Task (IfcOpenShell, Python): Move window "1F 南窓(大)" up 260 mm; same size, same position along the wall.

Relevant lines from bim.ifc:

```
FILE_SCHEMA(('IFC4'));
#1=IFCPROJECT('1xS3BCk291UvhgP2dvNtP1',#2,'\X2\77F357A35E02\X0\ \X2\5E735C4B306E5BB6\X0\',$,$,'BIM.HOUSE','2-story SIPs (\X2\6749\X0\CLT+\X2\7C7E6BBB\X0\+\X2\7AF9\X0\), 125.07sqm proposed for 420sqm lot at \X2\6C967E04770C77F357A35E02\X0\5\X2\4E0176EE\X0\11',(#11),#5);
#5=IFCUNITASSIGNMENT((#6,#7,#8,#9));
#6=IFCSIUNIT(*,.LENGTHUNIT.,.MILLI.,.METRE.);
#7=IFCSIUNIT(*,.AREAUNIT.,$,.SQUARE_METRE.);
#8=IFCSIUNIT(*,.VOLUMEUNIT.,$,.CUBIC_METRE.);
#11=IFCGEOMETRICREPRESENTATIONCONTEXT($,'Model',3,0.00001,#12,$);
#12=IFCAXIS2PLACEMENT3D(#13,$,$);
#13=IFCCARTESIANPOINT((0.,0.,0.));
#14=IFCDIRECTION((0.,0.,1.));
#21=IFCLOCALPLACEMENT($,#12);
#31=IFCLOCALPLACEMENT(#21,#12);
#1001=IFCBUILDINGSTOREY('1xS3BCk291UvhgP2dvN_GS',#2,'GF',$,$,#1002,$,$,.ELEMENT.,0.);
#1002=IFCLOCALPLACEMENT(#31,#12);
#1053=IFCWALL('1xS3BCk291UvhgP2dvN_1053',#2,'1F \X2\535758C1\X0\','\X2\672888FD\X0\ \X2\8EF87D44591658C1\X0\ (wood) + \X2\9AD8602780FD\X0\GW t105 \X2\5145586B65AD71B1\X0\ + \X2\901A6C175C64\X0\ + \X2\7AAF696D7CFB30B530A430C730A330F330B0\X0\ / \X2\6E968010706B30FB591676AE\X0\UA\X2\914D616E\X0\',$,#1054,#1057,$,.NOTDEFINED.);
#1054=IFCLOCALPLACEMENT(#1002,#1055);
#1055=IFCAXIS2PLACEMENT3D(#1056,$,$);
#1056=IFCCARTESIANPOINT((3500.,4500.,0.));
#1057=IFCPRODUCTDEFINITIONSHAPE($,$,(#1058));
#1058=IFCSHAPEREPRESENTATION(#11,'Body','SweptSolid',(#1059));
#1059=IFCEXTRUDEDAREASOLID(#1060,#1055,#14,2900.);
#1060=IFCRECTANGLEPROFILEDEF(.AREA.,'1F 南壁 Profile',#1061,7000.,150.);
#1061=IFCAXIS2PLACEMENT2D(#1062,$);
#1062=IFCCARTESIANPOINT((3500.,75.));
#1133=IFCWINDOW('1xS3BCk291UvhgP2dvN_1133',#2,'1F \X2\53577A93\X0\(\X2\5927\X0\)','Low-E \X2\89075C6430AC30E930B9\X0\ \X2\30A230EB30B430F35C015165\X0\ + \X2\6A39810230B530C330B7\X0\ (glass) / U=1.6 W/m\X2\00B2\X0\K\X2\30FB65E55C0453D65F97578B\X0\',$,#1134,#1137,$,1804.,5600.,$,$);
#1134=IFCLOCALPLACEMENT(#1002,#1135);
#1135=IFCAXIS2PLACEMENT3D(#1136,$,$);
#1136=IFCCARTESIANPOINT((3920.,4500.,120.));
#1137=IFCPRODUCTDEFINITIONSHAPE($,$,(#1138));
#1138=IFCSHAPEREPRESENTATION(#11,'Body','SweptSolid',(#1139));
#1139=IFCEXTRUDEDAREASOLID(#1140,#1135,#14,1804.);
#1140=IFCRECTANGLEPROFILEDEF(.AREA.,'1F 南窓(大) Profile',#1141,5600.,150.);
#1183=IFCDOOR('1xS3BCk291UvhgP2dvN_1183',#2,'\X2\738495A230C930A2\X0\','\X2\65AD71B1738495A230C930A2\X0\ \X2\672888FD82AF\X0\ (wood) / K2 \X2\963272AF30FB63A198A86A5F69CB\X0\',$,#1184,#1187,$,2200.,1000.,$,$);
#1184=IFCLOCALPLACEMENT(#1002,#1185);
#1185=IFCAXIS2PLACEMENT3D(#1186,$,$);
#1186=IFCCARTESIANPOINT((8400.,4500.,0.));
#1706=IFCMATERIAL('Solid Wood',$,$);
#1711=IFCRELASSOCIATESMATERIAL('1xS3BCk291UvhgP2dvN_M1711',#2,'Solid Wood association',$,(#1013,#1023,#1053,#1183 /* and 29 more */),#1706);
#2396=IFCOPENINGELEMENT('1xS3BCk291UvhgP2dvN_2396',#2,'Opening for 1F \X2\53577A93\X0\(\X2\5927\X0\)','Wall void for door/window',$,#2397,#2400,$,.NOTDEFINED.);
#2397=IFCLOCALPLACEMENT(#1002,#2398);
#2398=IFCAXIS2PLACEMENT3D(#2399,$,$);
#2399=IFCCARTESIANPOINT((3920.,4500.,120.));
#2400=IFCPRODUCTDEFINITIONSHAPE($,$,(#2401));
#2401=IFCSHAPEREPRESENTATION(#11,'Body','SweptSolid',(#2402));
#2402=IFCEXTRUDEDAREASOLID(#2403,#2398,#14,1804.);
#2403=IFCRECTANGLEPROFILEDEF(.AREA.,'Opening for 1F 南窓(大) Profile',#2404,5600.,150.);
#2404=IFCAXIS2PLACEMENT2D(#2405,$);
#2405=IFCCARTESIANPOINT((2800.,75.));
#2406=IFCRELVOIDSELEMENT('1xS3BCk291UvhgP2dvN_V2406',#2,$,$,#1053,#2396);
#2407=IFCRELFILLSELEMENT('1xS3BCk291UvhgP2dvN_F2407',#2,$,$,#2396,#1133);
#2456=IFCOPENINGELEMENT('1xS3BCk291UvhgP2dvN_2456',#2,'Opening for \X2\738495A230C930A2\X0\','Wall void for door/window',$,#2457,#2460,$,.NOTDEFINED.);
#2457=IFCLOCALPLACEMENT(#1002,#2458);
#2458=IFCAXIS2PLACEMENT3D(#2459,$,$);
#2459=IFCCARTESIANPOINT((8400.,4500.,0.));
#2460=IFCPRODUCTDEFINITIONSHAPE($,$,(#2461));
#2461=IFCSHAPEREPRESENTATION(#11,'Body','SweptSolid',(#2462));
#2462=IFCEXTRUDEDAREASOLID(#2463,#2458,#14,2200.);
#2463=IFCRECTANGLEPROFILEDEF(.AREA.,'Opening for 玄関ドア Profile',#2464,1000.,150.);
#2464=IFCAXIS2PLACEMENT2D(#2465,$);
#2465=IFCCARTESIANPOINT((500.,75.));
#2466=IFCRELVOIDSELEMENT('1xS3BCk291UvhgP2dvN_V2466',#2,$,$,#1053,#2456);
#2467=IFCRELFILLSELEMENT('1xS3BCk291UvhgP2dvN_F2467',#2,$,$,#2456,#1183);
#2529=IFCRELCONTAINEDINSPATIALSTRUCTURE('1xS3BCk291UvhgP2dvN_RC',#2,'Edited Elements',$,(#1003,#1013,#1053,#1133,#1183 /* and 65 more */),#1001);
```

```python
import numpy as np
import ifcopenshell
import ifcopenshell.api.geometry
import ifcopenshell.util.placement
import ifcopenshell.util.unit

model = ifcopenshell.open("bim.ifc")
unit_scale = ifcopenshell.util.unit.calculate_unit_scale(model)

window = model.by_guid("1xS3BCk291UvhgP2dvN_1133")
opening = window.FillsVoids[0].RelatingOpeningElement
dz = 0.26 / unit_scale

shift = np.array([0.0, 0.0, dz])
# The window is not placed relative to its opening, so move both.
for product in (opening, window):
    matrix = ifcopenshell.util.placement.get_local_placement(product.ObjectPlacement)
    matrix[:3, 3] += shift
    ifcopenshell.api.geometry.edit_object_placement(model, product=product, matrix=matrix, is_si=False)

print(f"moved by {dz * unit_scale:+.3f} m")

model.write("bim_edited.ifc")
```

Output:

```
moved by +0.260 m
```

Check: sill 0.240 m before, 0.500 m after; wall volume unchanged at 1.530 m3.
